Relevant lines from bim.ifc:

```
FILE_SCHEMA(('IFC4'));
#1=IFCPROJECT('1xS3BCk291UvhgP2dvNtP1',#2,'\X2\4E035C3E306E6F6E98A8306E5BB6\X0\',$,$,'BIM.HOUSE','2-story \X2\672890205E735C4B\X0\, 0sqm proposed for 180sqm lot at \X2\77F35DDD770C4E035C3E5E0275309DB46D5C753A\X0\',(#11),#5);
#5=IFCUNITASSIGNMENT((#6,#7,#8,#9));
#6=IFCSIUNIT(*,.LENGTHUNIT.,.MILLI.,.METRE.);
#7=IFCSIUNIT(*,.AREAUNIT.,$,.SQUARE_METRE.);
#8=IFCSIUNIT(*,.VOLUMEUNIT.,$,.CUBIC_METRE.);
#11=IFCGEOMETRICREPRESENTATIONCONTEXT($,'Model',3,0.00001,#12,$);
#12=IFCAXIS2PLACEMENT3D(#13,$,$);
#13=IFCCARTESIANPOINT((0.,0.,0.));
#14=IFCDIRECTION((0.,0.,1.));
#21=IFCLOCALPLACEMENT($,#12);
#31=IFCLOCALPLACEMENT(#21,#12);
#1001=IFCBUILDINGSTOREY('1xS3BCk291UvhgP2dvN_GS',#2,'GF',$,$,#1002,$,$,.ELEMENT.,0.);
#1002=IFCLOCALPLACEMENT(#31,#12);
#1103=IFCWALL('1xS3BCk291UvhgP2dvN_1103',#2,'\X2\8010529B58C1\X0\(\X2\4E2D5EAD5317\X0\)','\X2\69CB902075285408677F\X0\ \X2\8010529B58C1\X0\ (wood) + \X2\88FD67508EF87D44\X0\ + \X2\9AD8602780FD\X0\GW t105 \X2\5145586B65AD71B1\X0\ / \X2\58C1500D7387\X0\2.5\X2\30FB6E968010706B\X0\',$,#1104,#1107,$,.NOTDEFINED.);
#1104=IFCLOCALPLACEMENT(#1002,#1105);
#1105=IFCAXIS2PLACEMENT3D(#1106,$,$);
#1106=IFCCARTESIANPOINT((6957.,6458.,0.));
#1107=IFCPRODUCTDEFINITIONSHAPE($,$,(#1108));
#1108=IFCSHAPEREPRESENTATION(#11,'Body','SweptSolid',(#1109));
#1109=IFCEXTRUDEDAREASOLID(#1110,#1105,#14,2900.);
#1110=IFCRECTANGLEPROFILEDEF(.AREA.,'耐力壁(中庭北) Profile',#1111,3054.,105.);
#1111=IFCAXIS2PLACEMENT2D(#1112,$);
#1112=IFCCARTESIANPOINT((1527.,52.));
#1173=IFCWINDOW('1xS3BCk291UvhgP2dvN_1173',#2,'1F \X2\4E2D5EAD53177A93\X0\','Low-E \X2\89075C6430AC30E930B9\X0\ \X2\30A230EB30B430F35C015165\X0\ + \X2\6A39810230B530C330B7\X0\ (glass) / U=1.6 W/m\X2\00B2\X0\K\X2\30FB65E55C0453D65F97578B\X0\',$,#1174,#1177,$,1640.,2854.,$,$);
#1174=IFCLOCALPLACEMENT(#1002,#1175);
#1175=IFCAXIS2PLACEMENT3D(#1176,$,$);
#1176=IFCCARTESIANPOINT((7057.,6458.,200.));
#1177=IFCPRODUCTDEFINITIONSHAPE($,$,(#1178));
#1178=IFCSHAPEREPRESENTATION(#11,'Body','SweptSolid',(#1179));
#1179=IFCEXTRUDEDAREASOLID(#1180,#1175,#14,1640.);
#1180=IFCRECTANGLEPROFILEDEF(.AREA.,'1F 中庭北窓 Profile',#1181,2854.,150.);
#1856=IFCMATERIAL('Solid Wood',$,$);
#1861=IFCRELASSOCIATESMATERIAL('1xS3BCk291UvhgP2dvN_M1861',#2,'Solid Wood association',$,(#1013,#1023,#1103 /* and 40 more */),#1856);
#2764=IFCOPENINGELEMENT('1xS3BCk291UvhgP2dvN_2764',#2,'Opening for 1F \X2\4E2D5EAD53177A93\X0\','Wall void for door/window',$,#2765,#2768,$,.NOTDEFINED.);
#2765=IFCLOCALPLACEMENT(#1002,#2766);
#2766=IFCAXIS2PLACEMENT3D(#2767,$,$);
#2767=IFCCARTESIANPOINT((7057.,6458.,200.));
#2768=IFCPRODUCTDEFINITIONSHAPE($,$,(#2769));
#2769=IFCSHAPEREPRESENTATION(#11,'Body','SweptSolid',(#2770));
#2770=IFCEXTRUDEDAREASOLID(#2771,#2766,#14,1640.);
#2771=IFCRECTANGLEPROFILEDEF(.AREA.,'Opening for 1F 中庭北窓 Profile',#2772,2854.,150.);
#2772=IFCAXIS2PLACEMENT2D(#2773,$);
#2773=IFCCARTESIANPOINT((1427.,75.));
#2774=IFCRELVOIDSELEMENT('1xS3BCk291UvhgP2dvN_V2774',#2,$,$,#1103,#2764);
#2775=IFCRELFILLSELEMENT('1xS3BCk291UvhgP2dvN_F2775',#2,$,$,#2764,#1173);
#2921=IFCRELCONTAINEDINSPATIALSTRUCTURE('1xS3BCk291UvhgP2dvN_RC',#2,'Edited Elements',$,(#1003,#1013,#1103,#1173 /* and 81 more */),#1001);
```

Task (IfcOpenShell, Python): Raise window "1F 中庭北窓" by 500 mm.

```python
import numpy as np
import ifcopenshell
import ifcopenshell.api.geometry
import ifcopenshell.util.placement
import ifcopenshell.util.unit

model = ifcopenshell.open("bim.ifc")
unit_scale = ifcopenshell.util.unit.calculate_unit_scale(model)

window = model.by_id(1173)
opening = window.FillsVoids[0].RelatingOpeningElement
dz = 0.5 / unit_scale

shift = np.array([0.0, 0.0, dz])
# The window is not placed relative to its opening, so move both.
for product in (opening, window):
    matrix = ifcopenshell.util.placement.get_local_placement(product.ObjectPlacement)
    matrix[:3, 3] += shift
    ifcopenshell.api.geometry.edit_object_placement(model, product=product, matrix=matrix, is_si=False)

print(f"moved by {dz * unit_scale:+.3f} m")

model.write("bim_updated.ifc")
```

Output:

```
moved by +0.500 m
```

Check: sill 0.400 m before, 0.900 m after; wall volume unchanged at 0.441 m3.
